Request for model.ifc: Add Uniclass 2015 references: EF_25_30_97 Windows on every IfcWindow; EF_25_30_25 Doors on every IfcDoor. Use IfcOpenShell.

First a look at what the model holds.

```python
import ifcopenshell

model = ifcopenshell.open("model.ifc")
print(model.schema)
print("classifications:", [c.Name for c in model.by_type("IfcClassification")])
for ifc_class in ("IfcDoor", "IfcRoof", "IfcStair", "IfcWall", "IfcWindow"):
    print(ifc_class, len(model.by_type(ifc_class)))
```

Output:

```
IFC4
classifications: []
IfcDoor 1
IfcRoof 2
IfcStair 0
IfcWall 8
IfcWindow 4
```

```python
import ifcopenshell
import ifcopenshell.api.classification

model = ifcopenshell.open("model.ifc")

system = ifcopenshell.api.classification.add_classification(model, classification="Uniclass 2015")

codes = {
    "IfcWindow": ("EF_25_30_97", "Windows"),
    "IfcDoor": ("EF_25_30_25", "Doors"),
}
for ifc_class, (code, name) in codes.items():
    products = model.by_type(ifc_class)
    ifcopenshell.api.classification.add_reference(
        model, products=products, classification=system, identification=code, name=name
    )
    print(code, len(products))

model.write("model_updated.ifc")
```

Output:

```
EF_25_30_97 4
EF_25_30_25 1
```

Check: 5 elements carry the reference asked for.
